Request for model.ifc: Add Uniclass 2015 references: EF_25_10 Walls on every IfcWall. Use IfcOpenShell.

First a look at what the model holds.

```python
import ifcopenshell

model = ifcopenshell.open("model.ifc")
print(model.schema)
print("classifications:", [c.Name for c in model.by_type("IfcClassification")])
for ifc_class in ("IfcDoor", "IfcRoof", "IfcStair", "IfcWall", "IfcWindow"):
    print(ifc_class, len(model.by_type(ifc_class)))
```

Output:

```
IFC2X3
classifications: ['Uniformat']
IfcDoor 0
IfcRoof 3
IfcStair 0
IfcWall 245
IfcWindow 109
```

```python
import ifcopenshell
import ifcopenshell.api.classification

model = ifcopenshell.open("model.ifc")

# IFC2X3 requires Source and Edition and has no link from the project to the system.
system = model.create_entity("IfcClassification", Source="NBS", Edition="2015", Name="Uniclass 2015")

codes = {
    "IfcWall": ("EF_25_10", "Walls"),
}
for ifc_class, (code, name) in codes.items():
    products = model.by_type(ifc_class)
    ifcopenshell.api.classification.add_reference(
        model, products=products, classification=system, identification=code, name=name
    )
    print(code, len(products))

model.write("model-out.ifc")
```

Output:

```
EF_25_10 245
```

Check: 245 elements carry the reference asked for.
